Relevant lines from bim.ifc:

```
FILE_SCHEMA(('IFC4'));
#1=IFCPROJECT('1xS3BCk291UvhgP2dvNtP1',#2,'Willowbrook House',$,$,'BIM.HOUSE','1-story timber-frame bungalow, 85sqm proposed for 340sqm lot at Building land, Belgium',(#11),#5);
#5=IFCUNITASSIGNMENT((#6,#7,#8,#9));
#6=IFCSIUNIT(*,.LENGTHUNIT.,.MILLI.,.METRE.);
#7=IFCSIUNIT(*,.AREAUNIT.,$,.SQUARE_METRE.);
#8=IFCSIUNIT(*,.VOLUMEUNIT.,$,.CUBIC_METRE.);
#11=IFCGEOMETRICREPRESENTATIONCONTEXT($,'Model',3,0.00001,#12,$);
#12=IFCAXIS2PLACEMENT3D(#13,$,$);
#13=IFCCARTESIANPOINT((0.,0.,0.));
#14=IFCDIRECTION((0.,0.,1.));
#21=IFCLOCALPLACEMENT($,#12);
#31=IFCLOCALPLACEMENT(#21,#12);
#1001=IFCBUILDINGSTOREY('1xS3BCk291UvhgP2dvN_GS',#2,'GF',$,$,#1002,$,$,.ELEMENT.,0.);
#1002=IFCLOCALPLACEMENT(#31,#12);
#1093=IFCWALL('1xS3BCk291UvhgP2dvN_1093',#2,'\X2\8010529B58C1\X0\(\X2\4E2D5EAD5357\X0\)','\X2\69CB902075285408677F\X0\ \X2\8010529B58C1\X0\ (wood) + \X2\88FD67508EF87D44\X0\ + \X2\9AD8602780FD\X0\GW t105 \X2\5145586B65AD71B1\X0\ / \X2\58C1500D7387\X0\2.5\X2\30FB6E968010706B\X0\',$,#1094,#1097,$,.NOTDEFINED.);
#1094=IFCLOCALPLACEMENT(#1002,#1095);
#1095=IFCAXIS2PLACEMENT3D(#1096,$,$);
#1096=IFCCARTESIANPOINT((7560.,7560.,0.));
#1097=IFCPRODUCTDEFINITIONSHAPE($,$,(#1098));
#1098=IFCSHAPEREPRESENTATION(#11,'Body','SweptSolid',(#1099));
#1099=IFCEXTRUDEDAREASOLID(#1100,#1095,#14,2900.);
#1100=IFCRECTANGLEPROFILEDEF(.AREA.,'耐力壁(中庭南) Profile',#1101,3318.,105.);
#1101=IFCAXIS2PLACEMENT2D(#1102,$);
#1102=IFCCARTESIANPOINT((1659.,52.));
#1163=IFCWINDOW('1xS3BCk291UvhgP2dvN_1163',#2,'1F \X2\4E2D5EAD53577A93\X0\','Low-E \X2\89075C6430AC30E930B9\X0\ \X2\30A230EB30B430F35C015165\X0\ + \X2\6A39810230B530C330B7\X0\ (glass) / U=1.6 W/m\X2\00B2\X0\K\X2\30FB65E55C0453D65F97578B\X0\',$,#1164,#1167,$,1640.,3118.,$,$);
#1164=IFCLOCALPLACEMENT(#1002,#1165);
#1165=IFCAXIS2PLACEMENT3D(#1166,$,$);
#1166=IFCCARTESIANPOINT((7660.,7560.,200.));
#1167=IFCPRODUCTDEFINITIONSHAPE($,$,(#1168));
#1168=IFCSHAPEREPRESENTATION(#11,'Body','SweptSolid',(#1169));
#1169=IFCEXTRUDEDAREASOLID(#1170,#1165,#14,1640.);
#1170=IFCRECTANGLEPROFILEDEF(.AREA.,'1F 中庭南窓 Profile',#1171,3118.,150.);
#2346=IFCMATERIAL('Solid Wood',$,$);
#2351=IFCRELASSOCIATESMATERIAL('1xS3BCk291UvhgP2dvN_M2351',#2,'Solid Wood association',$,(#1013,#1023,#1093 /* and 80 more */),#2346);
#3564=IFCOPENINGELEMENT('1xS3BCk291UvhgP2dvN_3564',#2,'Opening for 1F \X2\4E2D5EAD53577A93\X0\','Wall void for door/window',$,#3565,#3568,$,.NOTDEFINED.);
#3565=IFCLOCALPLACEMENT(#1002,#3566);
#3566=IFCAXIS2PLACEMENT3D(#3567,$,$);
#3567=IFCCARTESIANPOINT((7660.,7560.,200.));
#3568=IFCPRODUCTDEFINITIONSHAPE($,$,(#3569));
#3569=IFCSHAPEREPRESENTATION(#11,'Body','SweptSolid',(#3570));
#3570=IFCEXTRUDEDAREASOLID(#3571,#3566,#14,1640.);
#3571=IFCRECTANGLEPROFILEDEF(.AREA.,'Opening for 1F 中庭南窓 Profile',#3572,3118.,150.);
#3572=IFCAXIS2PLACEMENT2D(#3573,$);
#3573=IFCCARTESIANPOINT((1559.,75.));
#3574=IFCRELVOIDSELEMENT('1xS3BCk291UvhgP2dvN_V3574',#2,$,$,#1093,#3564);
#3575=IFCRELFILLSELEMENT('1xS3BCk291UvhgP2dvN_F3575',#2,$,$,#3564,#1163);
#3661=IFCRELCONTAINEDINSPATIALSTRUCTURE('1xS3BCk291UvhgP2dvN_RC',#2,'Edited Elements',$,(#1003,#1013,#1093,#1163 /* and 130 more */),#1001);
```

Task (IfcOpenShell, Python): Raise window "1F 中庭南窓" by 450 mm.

```python
import numpy as np
import ifcopenshell
import ifcopenshell.api.geometry
import ifcopenshell.util.placement
import ifcopenshell.util.unit

model = ifcopenshell.open("bim.ifc")
unit_scale = ifcopenshell.util.unit.calculate_unit_scale(model)

window = model.by_guid("1xS3BCk291UvhgP2dvN_1163")
opening = window.FillsVoids[0].RelatingOpeningElement
dz = 450.0

shift = np.array([0.0, 0.0, dz])
# The window is not placed relative to its opening, so move both.
for product in (opening, window):
    matrix = ifcopenshell.util.placement.get_local_placement(product.ObjectPlacement)
    matrix[:3, 3] += shift
    ifcopenshell.api.geometry.edit_object_placement(model, product=product, matrix=matrix, is_si=False)

print(f"moved by {dz * unit_scale:+.3f} m")

model.write("bim_rev.ifc")
```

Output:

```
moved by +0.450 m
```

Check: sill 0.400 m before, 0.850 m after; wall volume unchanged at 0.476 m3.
